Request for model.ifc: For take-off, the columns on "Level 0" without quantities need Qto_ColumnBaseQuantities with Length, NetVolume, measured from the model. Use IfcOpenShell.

First a look at what the model holds.

```python
import ifcopenshell
import ifcopenshell.util.element
import ifcopenshell.util.unit

model = ifcopenshell.open("model.ifc")
print(model.schema)
for unit_type in ("LENGTHUNIT", "AREAUNIT", "VOLUMEUNIT"):
    print(unit_type, ifcopenshell.util.unit.calculate_unit_scale(model, unit_type))
storey = next(s for s in model.by_type("IfcBuildingStorey") if s.Name == "Level 0")
columns = [e for e in ifcopenshell.util.element.get_decomposition(storey) if e.is_a("IfcColumn")]
for e in sorted(columns, key=lambda e: e.id()):
    print(e.id(), e.is_a(), e.Name, list(ifcopenshell.util.element.get_psets(e, qtos_only=True)), sep=" | ")
```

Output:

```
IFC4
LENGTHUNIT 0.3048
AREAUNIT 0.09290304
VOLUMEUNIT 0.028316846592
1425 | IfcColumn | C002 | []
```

```python
import ifcopenshell
import ifcopenshell.api.pset
import ifcopenshell.geom
import ifcopenshell.util.element
import ifcopenshell.util.shape
import ifcopenshell.util.unit

model = ifcopenshell.open("model.ifc")
unit_scale = ifcopenshell.util.unit.calculate_unit_scale(model)
volume_scale = ifcopenshell.util.unit.calculate_unit_scale(model, "VOLUMEUNIT")
settings = ifcopenshell.geom.settings()

storey = next(s for s in model.by_type("IfcBuildingStorey") if s.Name == "Level 0")
columns = [e for e in ifcopenshell.util.element.get_decomposition(storey) if e.is_a("IfcColumn")]

for e in sorted(columns, key=lambda e: e.id()):
    if ifcopenshell.util.element.get_psets(e, qtos_only=True, should_inherit=False):
        continue
    # Geometry comes back in metres, in the element's own axes.
    shape = ifcopenshell.geom.create_shape(settings, e)
    values = {
        "Length": ifcopenshell.util.shape.get_z(shape.geometry) / unit_scale,
        "NetVolume": ifcopenshell.util.shape.get_volume(shape.geometry) / volume_scale,
    }
    qto = ifcopenshell.api.pset.add_qto(model, product=e, name="Qto_ColumnBaseQuantities")
    ifcopenshell.api.pset.edit_qto(model, qto=qto, properties=values)
    print(e.id(), {k: round(v, 3) for k, v in values.items()})

model.write("model-out.ifc")
```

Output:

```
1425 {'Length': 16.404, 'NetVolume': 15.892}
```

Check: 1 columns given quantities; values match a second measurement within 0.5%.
